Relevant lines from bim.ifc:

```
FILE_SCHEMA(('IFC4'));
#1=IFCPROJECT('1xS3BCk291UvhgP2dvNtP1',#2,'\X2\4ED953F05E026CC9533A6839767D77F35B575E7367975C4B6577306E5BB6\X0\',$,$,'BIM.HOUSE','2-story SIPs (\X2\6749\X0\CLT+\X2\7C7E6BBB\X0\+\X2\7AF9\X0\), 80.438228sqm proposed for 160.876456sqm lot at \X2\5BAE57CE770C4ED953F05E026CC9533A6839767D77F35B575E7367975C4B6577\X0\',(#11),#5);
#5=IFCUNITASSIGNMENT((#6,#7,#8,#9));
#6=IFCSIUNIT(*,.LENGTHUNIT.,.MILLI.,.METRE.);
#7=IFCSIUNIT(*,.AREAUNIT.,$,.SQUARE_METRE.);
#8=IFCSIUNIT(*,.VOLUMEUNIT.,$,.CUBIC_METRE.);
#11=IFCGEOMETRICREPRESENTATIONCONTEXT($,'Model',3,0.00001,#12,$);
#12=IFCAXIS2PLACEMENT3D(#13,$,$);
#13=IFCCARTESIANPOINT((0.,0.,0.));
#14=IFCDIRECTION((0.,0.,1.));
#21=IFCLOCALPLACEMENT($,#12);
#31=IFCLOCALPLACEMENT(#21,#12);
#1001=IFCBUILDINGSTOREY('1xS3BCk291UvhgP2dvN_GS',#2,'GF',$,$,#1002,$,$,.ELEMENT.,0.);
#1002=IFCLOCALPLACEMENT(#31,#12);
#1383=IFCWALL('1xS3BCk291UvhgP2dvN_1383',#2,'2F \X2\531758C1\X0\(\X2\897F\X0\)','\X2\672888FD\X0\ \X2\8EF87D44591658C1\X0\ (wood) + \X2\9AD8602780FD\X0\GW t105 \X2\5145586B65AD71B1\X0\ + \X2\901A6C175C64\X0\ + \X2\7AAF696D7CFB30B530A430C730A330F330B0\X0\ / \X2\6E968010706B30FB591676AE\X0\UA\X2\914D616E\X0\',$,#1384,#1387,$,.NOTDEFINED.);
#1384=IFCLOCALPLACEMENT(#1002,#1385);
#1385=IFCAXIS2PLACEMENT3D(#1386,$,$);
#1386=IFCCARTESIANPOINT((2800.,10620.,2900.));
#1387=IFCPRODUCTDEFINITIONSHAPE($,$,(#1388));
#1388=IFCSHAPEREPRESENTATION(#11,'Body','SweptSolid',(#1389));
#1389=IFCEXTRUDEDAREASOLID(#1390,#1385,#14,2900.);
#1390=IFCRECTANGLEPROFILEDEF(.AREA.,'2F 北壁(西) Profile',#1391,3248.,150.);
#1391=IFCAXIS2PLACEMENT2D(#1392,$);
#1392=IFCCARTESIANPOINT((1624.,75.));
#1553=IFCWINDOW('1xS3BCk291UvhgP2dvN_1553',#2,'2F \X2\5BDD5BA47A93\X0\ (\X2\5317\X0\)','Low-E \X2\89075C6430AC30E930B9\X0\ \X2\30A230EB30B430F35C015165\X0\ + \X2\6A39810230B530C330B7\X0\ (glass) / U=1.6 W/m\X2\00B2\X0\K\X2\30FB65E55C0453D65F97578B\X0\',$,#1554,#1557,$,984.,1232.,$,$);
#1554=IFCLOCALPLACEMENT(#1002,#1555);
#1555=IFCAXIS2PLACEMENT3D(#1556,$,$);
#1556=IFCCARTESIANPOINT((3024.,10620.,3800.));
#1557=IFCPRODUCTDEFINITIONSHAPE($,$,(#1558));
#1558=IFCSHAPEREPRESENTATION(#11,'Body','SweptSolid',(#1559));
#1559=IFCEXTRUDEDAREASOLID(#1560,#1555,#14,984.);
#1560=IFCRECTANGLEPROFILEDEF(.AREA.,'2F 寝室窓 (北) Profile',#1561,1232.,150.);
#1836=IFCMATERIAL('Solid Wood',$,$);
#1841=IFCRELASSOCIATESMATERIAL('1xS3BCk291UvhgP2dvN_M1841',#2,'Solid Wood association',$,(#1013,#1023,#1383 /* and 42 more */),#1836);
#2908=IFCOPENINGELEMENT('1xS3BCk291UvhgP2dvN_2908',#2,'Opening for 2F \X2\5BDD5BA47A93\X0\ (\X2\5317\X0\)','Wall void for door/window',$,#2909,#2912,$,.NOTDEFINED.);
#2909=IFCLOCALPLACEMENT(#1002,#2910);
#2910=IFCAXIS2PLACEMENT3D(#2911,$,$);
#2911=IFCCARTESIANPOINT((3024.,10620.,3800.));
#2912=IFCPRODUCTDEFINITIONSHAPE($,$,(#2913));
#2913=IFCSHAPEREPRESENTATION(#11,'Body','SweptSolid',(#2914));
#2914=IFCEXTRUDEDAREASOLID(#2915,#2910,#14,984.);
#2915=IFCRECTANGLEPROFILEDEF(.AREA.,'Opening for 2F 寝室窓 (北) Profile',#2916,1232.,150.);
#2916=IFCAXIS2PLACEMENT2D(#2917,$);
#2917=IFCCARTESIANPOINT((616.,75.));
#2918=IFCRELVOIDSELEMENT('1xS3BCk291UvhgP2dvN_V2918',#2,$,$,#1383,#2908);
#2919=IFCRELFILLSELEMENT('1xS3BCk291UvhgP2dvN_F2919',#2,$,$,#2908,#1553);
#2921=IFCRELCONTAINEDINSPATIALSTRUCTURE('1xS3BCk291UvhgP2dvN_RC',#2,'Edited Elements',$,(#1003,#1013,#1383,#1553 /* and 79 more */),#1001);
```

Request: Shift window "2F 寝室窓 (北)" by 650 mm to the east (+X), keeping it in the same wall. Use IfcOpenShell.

```python
import ifcopenshell
import ifcopenshell.api.geometry
import ifcopenshell.util.placement
import ifcopenshell.util.unit

model = ifcopenshell.open("bim.ifc")
unit_scale = ifcopenshell.util.unit.calculate_unit_scale(model)

window = model.by_guid("1xS3BCk291UvhgP2dvN_1553")
opening = window.FillsVoids[0].RelatingOpeningElement
wall = opening.VoidsElements[0].RelatingBuildingElement

wall_matrix = ifcopenshell.util.placement.get_local_placement(wall.ObjectPlacement)
shift = wall_matrix[:3, 0] * 0.65 / unit_scale
before = ifcopenshell.util.placement.get_local_placement(window.ObjectPlacement)[:3, 3].copy()

# The window is not placed relative to its opening, so move both.
for product in (opening, window):
    matrix = ifcopenshell.util.placement.get_local_placement(product.ObjectPlacement)
    matrix[:3, 3] += shift
    ifcopenshell.api.geometry.edit_object_placement(model, product=product, matrix=matrix, is_si=False)

after = ifcopenshell.util.placement.get_local_placement(window.ObjectPlacement)[:3, 3]
print("window moved by", (after - before).round(3) + 0.0)

model.write("bim_updated.ifc")
```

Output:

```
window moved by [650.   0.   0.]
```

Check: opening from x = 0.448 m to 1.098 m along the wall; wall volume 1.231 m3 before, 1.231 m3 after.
